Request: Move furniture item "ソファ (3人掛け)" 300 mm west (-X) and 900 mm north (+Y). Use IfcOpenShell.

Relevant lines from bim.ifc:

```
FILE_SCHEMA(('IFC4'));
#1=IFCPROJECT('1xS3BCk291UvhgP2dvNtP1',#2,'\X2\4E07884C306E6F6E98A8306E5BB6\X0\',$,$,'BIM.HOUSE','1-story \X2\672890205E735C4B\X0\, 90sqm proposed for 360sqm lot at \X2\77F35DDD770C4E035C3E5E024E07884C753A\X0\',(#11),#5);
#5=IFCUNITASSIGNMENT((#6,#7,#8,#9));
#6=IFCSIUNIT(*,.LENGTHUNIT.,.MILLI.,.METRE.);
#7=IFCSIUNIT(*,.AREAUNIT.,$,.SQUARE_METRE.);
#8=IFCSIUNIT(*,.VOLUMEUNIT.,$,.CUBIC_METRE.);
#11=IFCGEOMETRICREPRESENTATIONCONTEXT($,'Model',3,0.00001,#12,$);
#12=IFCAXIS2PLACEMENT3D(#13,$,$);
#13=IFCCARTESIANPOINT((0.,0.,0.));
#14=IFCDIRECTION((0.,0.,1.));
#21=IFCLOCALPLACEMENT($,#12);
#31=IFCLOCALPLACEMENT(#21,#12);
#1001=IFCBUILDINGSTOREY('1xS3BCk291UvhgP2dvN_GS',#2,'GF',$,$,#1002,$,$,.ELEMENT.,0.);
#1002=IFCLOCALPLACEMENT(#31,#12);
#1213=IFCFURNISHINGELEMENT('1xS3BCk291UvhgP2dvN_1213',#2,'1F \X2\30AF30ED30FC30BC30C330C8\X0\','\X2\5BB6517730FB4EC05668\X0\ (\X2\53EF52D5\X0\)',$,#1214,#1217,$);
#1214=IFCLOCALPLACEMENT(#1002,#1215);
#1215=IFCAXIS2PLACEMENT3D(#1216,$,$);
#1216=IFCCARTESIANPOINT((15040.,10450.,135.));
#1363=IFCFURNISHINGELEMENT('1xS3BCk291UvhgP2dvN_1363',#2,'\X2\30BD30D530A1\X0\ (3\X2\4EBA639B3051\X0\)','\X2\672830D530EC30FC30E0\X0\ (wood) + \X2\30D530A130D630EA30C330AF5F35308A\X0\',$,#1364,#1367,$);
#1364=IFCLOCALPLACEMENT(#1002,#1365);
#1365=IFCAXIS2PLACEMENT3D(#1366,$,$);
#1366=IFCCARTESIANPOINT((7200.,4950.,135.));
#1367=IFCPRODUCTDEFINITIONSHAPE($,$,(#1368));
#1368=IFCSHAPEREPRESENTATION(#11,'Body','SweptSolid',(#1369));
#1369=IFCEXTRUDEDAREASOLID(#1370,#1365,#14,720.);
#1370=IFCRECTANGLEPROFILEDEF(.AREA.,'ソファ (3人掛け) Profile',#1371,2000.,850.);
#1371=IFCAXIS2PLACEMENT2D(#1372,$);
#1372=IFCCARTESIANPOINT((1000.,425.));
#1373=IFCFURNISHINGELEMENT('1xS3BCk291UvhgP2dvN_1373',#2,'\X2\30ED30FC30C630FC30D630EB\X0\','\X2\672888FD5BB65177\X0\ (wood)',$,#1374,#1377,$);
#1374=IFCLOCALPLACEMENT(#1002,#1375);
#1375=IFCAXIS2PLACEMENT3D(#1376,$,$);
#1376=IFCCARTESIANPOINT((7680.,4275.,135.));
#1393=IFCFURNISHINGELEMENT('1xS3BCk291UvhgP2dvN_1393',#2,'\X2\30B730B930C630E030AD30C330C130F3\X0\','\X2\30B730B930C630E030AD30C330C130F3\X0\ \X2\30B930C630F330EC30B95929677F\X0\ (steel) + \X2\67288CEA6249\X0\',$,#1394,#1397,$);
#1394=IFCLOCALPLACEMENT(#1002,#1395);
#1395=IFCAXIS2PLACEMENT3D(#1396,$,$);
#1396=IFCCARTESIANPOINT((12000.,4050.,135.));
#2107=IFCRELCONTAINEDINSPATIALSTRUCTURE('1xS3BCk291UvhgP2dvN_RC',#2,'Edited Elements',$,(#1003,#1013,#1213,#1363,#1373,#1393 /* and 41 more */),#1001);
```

```python
import ifcopenshell
import ifcopenshell.api.geometry
import ifcopenshell.util.placement
import ifcopenshell.util.unit

model = ifcopenshell.open("bim.ifc")
unit_scale = ifcopenshell.util.unit.calculate_unit_scale(model)

item = model.by_guid("1xS3BCk291UvhgP2dvN_1363")
matrix = ifcopenshell.util.placement.get_local_placement(item.ObjectPlacement)
matrix[0, 3] -= 0.3 / unit_scale
matrix[1, 3] += 0.9 / unit_scale
ifcopenshell.api.geometry.edit_object_placement(model, product=item, matrix=matrix, is_si=False)

print(ifcopenshell.util.placement.get_local_placement(item.ObjectPlacement).round(3) + 0.0)

model.write("bim_updated.ifc")
```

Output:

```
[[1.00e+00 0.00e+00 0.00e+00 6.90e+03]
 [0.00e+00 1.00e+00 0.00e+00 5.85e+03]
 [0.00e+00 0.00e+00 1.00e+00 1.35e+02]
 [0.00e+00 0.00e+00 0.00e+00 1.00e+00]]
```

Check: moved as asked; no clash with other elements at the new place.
